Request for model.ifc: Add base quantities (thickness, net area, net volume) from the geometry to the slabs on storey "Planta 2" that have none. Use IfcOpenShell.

First a look at what the model holds.

```python
import ifcopenshell
import ifcopenshell.util.element
import ifcopenshell.util.unit

model = ifcopenshell.open("model.ifc")
print(model.schema)
for unit_type in ("LENGTHUNIT", "AREAUNIT", "VOLUMEUNIT"):
    print(unit_type, ifcopenshell.util.unit.calculate_unit_scale(model, unit_type))
storey = next(s for s in model.by_type("IfcBuildingStorey") if s.Name == "Planta 2")
slabs = [e for e in ifcopenshell.util.element.get_decomposition(storey) if e.is_a("IfcSlab")]
for e in sorted(slabs, key=lambda e: e.id()):
    print(e.id(), e.is_a(), e.Name, list(ifcopenshell.util.element.get_psets(e, qtos_only=True)), sep=" | ")
```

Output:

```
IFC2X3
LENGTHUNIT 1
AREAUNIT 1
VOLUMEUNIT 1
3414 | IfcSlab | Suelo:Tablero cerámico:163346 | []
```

```python
import ifcopenshell
import ifcopenshell.api.pset
import ifcopenshell.geom
import ifcopenshell.util.element
import ifcopenshell.util.shape
import ifcopenshell.util.unit

model = ifcopenshell.open("model.ifc")
unit_scale = ifcopenshell.util.unit.calculate_unit_scale(model)
area_scale = ifcopenshell.util.unit.calculate_unit_scale(model, "AREAUNIT")
volume_scale = ifcopenshell.util.unit.calculate_unit_scale(model, "VOLUMEUNIT")
settings = ifcopenshell.geom.settings()

storey = next(s for s in model.by_type("IfcBuildingStorey") if s.Name == "Planta 2")
slabs = [e for e in ifcopenshell.util.element.get_decomposition(storey) if e.is_a("IfcSlab")]

for e in sorted(slabs, key=lambda e: e.id()):
    if ifcopenshell.util.element.get_psets(e, qtos_only=True, should_inherit=False):
        continue
    # Geometry comes back in metres, in the element's own axes.
    shape = ifcopenshell.geom.create_shape(settings, e)
    values = {
        "Width": ifcopenshell.util.shape.get_z(shape.geometry) / unit_scale,
        "NetArea": ifcopenshell.util.shape.get_footprint_area(shape.geometry) / area_scale,
        "NetVolume": ifcopenshell.util.shape.get_volume(shape.geometry) / volume_scale,
    }
    qto = ifcopenshell.api.pset.add_qto(model, product=e, name="BaseQuantities")
    ifcopenshell.api.pset.edit_qto(model, qto=qto, properties=values)
    print(e.id(), {k: round(v, 3) for k, v in values.items()})

model.write("model_v2.ifc")
```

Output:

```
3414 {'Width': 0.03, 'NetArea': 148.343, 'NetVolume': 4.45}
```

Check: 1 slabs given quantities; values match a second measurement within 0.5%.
